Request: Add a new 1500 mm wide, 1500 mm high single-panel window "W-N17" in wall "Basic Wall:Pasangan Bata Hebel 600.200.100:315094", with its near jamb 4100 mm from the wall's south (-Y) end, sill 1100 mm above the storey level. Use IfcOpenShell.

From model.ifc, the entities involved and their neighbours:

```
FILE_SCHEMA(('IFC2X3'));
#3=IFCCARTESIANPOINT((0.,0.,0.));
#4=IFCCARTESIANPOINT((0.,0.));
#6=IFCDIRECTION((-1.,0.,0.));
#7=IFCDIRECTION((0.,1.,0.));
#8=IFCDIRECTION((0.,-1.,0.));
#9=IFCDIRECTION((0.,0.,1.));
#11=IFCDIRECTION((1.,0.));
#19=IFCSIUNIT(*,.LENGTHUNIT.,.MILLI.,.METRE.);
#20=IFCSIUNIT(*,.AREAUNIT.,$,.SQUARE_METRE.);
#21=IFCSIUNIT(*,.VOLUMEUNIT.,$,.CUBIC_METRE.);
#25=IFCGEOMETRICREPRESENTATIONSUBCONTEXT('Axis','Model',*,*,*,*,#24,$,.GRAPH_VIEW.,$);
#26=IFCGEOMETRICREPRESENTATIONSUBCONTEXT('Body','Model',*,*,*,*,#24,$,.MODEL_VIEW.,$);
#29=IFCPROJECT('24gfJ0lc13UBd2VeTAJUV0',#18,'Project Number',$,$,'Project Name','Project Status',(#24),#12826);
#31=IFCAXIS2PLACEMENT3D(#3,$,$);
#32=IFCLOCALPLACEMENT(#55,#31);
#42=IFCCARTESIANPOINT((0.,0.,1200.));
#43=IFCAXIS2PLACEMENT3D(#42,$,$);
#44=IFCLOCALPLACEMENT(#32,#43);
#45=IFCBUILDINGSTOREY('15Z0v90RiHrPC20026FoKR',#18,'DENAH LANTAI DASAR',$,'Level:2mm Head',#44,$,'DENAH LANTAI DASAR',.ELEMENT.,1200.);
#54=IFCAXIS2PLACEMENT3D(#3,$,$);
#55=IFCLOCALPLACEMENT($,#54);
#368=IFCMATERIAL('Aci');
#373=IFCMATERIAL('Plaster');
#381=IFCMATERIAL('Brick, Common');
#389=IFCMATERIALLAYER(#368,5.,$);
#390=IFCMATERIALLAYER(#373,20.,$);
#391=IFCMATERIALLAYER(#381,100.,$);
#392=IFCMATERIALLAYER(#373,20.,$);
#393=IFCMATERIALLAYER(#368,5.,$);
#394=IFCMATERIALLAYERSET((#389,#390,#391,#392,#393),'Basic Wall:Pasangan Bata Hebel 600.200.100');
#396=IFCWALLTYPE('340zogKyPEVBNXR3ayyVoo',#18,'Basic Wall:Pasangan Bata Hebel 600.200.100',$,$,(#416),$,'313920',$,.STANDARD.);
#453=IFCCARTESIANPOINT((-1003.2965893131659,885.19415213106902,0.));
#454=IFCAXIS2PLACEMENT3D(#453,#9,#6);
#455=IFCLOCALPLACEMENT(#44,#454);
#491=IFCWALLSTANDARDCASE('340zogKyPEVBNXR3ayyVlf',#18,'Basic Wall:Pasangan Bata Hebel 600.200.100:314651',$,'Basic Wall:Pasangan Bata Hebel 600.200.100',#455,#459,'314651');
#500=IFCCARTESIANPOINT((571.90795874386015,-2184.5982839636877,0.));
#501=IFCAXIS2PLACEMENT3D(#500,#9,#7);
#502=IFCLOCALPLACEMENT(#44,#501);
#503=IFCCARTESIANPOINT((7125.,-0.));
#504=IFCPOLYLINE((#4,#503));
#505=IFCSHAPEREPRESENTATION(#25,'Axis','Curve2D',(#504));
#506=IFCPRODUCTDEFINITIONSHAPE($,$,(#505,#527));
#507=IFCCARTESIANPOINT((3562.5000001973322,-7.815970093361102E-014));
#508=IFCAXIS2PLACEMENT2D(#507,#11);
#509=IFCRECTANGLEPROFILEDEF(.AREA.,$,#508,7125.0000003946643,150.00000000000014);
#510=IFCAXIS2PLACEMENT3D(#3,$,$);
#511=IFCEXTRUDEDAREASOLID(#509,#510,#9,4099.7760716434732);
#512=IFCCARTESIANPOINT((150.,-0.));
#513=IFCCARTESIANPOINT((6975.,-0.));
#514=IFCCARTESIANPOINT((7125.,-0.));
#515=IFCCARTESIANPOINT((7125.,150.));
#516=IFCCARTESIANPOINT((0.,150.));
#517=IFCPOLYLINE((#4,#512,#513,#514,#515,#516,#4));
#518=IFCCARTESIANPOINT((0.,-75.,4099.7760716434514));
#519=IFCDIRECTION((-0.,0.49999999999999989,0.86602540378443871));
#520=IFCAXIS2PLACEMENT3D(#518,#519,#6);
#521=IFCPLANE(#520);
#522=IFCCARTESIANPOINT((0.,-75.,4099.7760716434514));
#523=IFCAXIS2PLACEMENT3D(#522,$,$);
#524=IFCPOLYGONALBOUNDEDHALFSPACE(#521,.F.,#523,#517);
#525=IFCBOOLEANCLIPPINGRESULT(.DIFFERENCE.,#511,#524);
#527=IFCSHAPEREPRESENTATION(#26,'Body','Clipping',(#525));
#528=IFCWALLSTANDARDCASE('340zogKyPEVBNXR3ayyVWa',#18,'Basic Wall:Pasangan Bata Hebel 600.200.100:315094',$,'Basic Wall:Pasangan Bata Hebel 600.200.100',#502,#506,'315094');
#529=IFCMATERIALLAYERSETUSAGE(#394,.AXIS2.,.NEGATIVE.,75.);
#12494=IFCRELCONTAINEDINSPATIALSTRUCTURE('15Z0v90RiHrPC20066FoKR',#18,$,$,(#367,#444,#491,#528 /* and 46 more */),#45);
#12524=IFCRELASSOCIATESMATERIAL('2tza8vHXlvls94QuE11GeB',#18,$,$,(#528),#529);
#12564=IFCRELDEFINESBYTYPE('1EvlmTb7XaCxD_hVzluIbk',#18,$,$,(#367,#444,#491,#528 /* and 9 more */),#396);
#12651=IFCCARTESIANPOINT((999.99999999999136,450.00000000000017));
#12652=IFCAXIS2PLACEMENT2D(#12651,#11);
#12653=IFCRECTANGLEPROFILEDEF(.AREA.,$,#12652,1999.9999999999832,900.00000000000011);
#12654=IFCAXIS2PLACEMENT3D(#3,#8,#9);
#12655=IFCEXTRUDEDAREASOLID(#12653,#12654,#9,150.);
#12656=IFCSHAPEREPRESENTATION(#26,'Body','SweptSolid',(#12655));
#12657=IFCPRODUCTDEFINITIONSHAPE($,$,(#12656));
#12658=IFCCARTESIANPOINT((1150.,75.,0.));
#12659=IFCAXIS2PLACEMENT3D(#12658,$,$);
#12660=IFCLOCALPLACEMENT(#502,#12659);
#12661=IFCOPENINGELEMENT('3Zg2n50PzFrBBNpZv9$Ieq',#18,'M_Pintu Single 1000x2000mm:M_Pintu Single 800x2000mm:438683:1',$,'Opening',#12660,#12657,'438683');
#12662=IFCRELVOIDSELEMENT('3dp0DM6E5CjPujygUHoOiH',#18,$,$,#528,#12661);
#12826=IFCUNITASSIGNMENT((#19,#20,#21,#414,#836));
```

```python
import numpy as np
import ifcopenshell
import ifcopenshell.api.feature
import ifcopenshell.api.geometry
import ifcopenshell.api.root
import ifcopenshell.api.spatial
import ifcopenshell.api.type
import ifcopenshell.geom
import ifcopenshell.util.element
import ifcopenshell.util.placement
import ifcopenshell.util.representation
import ifcopenshell.util.shape
import ifcopenshell.util.unit

model = ifcopenshell.open("model.ifc")
unit_scale = ifcopenshell.util.unit.calculate_unit_scale(model)
settings = ifcopenshell.geom.settings()


def volume(element):
    """Net volume in cubic metres, openings subtracted."""
    shape = ifcopenshell.geom.create_shape(settings, element)
    return ifcopenshell.util.shape.get_volume(shape.geometry)


wall = model.by_guid("340zogKyPEVBNXR3ayyVWa")
storey = ifcopenshell.util.element.get_container(wall, ifc_class="IfcBuildingStorey")
context = ifcopenshell.util.representation.get_context(model, "Model", "Body", "MODEL_VIEW")
before = volume(wall)

width, height, from_end, sill = 1.5, 1.5, 4.1, 1.1  # metres

# The wall runs along its own X axis, and the end named is its -X end.
wall_shape = ifcopenshell.geom.create_shape(settings, wall)
x, y, z = ifcopenshell.util.shape.get_vertices(wall_shape.geometry).T
start = x.min() + from_end
face, thickness = float(y.min()), float(y.max() - y.min())
wall_matrix = ifcopenshell.util.placement.get_local_placement(wall.ObjectPlacement)
level = ifcopenshell.util.placement.get_local_placement(storey.ObjectPlacement)[2, 3]


def in_wall(x, y):
    """Placement at x, y metres in the wall's axes, at sill height."""
    matrix = wall_matrix.copy()
    matrix[:, 3] = wall_matrix @ np.array([x / unit_scale, y / unit_scale, 0.0, 1.0])
    matrix[2, 3] = level + sill / unit_scale
    return matrix


# Opening: a box that overshoots both wall faces by 50 mm.
opening = ifcopenshell.api.root.create_entity(model, ifc_class="IfcOpeningElement")
box = ifcopenshell.api.geometry.add_wall_representation(
    model, context=context, length=width, height=height, thickness=thickness + 0.1
)
ifcopenshell.api.geometry.assign_representation(model, product=opening, representation=box)
ifcopenshell.api.geometry.edit_object_placement(model, product=opening, matrix=in_wall(start, face - 0.05), is_si=False)
ifcopenshell.api.feature.add_feature(model, feature=opening, element=wall)

window = ifcopenshell.api.root.create_entity(model, ifc_class="IfcWindow", name="W-N17")
window.OverallWidth, window.OverallHeight = width / unit_scale, height / unit_scale
body = ifcopenshell.api.geometry.add_window_representation(
    model,
    context=context,
    overall_width=window.OverallWidth,
    overall_height=window.OverallHeight,
    partition_type="SINGLE_PANEL",
)
ifcopenshell.api.geometry.assign_representation(model, product=window, representation=body)
ifcopenshell.api.spatial.assign_container(model, products=[window], relating_structure=storey)
fills = ifcopenshell.api.feature.add_filling(model, opening=opening, element=window)
fills.OwnerHistory = window.OwnerHistory  # required in IFC2X3

# IFC2X3 keeps the operation on the window style.
style = ifcopenshell.api.root.create_entity(model, ifc_class="IfcWindowStyle", name="W-N17")
style.OperationType, style.ConstructionType = "SINGLE_PANEL", "NOTDEFINED"
style.ParameterTakesPrecedence = style.Sizeable = False
ifcopenshell.api.type.assign_type(model, related_objects=[window], relating_type=style)

# Centre the window in the wall's thickness.
ifcopenshell.api.geometry.edit_object_placement(model, product=window, matrix=in_wall(start, face), is_si=False)
window_shape = ifcopenshell.geom.create_shape(settings, window)
depth = ifcopenshell.util.shape.get_vertices(window_shape.geometry)[:, 1]
offset = face + thickness / 2 - (depth.min() + depth.max()) / 2
ifcopenshell.api.geometry.edit_object_placement(model, product=window, matrix=in_wall(start, offset), is_si=False)

after = volume(wall)

print(f"wall volume {before:.3f} -> {after:.3f} m3")

model.write("model-out.ifc")
```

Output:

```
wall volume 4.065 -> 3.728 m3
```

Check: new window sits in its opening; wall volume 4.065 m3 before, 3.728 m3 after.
